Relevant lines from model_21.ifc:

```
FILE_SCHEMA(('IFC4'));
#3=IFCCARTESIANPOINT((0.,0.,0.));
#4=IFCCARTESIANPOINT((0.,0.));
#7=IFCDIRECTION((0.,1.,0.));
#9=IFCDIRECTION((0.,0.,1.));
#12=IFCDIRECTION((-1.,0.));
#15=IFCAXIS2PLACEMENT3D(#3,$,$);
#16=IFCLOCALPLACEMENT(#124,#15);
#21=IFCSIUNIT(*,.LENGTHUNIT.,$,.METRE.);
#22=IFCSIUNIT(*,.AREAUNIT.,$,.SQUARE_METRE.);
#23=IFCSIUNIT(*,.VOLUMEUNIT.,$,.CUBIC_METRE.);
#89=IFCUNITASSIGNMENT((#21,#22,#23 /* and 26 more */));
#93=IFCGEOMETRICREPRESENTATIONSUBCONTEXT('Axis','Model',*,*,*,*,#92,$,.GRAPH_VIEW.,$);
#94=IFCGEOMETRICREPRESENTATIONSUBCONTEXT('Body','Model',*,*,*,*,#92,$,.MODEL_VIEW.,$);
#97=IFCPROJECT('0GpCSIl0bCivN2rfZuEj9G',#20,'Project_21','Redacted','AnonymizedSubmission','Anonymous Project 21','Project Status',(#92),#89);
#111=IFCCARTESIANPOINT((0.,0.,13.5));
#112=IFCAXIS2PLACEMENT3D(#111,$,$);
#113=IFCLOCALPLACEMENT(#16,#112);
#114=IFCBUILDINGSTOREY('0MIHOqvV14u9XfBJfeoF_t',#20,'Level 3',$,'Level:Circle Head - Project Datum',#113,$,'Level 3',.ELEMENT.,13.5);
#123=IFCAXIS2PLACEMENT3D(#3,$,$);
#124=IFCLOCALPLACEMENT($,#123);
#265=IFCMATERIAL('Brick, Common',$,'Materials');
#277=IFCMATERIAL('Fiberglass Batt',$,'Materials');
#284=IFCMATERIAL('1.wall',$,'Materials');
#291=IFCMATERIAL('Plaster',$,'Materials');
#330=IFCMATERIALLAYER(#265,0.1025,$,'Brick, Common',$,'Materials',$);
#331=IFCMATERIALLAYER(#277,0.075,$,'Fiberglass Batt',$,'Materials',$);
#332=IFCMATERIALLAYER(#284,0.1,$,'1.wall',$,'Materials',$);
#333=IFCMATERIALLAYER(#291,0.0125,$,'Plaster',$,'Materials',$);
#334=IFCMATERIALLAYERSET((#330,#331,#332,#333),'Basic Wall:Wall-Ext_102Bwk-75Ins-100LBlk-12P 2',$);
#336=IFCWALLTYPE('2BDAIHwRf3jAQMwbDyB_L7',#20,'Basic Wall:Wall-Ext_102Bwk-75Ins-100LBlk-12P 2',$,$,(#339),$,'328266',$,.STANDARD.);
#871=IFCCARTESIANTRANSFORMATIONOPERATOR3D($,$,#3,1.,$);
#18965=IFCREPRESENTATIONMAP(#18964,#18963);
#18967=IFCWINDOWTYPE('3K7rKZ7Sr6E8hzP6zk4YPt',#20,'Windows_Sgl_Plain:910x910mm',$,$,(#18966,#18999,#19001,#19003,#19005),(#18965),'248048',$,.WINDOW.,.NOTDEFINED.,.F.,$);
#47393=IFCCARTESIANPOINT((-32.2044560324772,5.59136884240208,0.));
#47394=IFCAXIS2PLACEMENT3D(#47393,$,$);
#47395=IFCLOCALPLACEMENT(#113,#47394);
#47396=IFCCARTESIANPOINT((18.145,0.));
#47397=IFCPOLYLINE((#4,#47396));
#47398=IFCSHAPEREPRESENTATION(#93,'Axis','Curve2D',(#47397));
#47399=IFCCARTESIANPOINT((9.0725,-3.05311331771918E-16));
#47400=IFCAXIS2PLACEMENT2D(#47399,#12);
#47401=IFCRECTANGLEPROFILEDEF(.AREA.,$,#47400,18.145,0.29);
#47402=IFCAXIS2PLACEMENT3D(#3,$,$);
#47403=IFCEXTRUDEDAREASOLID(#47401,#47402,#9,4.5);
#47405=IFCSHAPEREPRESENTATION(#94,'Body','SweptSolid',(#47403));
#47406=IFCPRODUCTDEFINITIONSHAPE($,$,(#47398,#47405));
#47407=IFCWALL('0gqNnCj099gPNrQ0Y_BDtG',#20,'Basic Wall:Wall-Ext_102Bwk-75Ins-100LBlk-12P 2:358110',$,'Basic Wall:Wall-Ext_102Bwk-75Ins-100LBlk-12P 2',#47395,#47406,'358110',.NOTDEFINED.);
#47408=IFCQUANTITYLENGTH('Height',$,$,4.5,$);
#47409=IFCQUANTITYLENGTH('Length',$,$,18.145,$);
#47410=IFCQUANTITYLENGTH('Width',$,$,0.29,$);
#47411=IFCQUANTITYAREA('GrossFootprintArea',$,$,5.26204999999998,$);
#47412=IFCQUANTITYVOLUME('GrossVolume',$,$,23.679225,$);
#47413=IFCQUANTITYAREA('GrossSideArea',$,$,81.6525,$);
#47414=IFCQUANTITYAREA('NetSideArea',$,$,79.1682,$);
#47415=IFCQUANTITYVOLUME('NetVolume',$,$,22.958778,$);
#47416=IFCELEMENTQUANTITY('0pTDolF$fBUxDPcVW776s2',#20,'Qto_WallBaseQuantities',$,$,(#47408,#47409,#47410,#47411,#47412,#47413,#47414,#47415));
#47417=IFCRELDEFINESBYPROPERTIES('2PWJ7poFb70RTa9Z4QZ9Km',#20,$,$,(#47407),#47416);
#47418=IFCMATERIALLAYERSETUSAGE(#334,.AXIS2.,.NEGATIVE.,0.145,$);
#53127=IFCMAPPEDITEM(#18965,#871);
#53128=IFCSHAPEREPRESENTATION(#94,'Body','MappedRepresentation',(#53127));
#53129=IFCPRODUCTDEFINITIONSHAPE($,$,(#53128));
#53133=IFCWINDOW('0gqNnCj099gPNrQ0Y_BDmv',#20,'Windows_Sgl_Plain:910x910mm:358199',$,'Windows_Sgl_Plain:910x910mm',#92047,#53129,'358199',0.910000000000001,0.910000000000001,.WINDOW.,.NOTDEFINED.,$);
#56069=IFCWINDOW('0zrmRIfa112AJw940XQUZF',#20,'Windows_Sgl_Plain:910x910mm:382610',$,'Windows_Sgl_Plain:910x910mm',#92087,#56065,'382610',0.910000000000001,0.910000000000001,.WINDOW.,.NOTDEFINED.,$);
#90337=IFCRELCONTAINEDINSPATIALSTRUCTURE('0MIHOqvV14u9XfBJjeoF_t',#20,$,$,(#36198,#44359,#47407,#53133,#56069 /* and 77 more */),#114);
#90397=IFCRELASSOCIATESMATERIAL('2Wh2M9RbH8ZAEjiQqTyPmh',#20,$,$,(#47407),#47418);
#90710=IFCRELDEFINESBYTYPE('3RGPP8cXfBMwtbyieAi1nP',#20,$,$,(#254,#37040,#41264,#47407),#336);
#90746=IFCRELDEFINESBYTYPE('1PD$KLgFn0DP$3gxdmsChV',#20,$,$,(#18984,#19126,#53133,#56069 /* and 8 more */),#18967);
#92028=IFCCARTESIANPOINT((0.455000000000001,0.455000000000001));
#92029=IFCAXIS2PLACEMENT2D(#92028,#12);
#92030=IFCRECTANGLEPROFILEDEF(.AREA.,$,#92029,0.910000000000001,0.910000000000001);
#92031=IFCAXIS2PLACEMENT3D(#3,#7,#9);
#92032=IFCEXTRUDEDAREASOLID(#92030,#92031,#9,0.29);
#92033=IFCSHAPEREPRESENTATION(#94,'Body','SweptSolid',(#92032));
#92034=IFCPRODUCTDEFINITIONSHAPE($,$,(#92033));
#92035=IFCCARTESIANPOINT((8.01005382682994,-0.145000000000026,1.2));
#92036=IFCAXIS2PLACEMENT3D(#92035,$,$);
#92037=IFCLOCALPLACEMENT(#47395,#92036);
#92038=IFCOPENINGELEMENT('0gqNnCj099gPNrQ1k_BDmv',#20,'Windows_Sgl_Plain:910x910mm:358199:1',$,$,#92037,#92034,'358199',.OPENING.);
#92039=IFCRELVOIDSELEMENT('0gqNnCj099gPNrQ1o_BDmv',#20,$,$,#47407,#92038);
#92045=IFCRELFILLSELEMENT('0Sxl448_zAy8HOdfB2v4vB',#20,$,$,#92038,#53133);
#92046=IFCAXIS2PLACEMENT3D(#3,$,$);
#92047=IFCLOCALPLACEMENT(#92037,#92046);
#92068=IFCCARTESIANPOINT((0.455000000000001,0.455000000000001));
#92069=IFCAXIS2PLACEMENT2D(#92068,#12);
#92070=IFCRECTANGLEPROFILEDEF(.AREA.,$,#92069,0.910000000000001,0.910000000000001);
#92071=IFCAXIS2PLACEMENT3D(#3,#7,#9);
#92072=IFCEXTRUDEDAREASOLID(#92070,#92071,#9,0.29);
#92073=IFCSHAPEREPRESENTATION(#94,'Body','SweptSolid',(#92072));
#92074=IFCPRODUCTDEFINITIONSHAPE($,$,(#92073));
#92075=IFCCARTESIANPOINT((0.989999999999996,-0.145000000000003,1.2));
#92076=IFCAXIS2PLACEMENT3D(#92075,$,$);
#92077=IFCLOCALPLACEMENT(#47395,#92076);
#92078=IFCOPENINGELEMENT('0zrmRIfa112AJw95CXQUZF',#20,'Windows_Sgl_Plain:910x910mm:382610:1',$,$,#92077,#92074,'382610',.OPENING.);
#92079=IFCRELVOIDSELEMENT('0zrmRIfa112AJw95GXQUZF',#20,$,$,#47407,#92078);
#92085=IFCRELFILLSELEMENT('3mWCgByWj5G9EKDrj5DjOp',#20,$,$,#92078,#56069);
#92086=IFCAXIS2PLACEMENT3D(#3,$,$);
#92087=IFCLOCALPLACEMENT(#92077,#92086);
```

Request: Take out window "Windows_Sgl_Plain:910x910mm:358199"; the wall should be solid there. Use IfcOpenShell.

```python
import ifcopenshell
import ifcopenshell.api.feature
import ifcopenshell.api.pset
import ifcopenshell.api.root
import ifcopenshell.geom
import ifcopenshell.util.element
import ifcopenshell.util.shape
import ifcopenshell.util.unit

model = ifcopenshell.open("model_21.ifc")
area_scale = ifcopenshell.util.unit.calculate_unit_scale(model, "AREAUNIT")
volume_scale = ifcopenshell.util.unit.calculate_unit_scale(model, "VOLUMEUNIT")
settings = ifcopenshell.geom.settings()


def volume(element):
    """Net volume in cubic metres, openings subtracted."""
    shape = ifcopenshell.geom.create_shape(settings, element)
    return ifcopenshell.util.shape.get_volume(shape.geometry)


window = model.by_guid("0gqNnCj099gPNrQ0Y_BDmv")
opening = window.FillsVoids[0].RelatingOpeningElement
wall = opening.VoidsElements[0].RelatingBuildingElement
before = volume(wall)

ifcopenshell.api.root.remove_product(model, product=window)
ifcopenshell.api.feature.remove_feature(model, feature=opening)

after = volume(wall)
thickness = 0.29  # wall thickness in metres

# Update the wall's stored quantities.
qto = model.by_id(ifcopenshell.util.element.get_pset(wall, "Qto_WallBaseQuantities", should_inherit=False)["id"])
ifcopenshell.api.pset.edit_qto(model, qto=qto, properties={
    "NetSideArea": after / thickness / area_scale,
    "NetVolume": after / volume_scale,
})

print(f"wall volume {before:.3f} -> {after:.3f} m3")

model.write("model_21_v2.ifc")
```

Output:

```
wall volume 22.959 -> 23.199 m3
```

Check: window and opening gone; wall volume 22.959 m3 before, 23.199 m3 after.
